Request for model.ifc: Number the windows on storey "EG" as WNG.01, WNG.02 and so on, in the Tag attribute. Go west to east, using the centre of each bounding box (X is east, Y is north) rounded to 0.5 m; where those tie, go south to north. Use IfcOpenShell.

First a look at what the model holds.

```python
import ifcopenshell
import ifcopenshell.util.element
import ifcopenshell.util.placement

model = ifcopenshell.open("model.ifc")
print(model.schema)
storey = next(s for s in model.by_type("IfcBuildingStorey") if s.Name == "EG")
windows = [e for e in ifcopenshell.util.element.get_decomposition(storey) if e.is_a("IfcWindow")]
for e in sorted(windows, key=lambda e: e.id()):
    origin = ifcopenshell.util.placement.get_local_placement(e.ObjectPlacement)[:3, 3]
    print(e.id(), e.Tag, e.Name, origin.round(2) + 0.0, sep=" | ")
```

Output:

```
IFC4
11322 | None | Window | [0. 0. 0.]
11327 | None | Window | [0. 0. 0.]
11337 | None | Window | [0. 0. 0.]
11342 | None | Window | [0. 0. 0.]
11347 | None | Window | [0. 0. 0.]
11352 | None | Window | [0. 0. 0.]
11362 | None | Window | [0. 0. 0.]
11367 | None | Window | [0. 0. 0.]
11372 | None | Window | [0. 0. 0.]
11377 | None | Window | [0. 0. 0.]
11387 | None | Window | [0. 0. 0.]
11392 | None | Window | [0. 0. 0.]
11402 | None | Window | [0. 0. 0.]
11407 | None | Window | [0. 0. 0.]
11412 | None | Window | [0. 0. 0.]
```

```python
import ifcopenshell
import ifcopenshell.geom
import ifcopenshell.util.element
import ifcopenshell.util.shape

model = ifcopenshell.open("model.ifc")
settings = ifcopenshell.geom.settings()
settings.set("use-world-coords", True)


def centre(element):
    shape = ifcopenshell.geom.create_shape(settings, element)
    return ifcopenshell.util.shape.get_bbox_centroid(shape.geometry)


storey = next(s for s in model.by_type("IfcBuildingStorey") if s.Name == "EG")
windows = [e for e in ifcopenshell.util.element.get_decomposition(storey) if e.is_a("IfcWindow")]

# Insertion points can sit at a corner or the storey origin, so sort by the geometry (in metres).
centres = {e: centre(e) for e in windows}
windows.sort(key=lambda e: (round(centres[e][0] / 0.5), centres[e][1]))

for i, e in enumerate(windows, start=1):
    number = f"WNG.{i:02d}"
    e.Tag = number
    print(e.id(), number)

model.write("model_rev.ifc")
```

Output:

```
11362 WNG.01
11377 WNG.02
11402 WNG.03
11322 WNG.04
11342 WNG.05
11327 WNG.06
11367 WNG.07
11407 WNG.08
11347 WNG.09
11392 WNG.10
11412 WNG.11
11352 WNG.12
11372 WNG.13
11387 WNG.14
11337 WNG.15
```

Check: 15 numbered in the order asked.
